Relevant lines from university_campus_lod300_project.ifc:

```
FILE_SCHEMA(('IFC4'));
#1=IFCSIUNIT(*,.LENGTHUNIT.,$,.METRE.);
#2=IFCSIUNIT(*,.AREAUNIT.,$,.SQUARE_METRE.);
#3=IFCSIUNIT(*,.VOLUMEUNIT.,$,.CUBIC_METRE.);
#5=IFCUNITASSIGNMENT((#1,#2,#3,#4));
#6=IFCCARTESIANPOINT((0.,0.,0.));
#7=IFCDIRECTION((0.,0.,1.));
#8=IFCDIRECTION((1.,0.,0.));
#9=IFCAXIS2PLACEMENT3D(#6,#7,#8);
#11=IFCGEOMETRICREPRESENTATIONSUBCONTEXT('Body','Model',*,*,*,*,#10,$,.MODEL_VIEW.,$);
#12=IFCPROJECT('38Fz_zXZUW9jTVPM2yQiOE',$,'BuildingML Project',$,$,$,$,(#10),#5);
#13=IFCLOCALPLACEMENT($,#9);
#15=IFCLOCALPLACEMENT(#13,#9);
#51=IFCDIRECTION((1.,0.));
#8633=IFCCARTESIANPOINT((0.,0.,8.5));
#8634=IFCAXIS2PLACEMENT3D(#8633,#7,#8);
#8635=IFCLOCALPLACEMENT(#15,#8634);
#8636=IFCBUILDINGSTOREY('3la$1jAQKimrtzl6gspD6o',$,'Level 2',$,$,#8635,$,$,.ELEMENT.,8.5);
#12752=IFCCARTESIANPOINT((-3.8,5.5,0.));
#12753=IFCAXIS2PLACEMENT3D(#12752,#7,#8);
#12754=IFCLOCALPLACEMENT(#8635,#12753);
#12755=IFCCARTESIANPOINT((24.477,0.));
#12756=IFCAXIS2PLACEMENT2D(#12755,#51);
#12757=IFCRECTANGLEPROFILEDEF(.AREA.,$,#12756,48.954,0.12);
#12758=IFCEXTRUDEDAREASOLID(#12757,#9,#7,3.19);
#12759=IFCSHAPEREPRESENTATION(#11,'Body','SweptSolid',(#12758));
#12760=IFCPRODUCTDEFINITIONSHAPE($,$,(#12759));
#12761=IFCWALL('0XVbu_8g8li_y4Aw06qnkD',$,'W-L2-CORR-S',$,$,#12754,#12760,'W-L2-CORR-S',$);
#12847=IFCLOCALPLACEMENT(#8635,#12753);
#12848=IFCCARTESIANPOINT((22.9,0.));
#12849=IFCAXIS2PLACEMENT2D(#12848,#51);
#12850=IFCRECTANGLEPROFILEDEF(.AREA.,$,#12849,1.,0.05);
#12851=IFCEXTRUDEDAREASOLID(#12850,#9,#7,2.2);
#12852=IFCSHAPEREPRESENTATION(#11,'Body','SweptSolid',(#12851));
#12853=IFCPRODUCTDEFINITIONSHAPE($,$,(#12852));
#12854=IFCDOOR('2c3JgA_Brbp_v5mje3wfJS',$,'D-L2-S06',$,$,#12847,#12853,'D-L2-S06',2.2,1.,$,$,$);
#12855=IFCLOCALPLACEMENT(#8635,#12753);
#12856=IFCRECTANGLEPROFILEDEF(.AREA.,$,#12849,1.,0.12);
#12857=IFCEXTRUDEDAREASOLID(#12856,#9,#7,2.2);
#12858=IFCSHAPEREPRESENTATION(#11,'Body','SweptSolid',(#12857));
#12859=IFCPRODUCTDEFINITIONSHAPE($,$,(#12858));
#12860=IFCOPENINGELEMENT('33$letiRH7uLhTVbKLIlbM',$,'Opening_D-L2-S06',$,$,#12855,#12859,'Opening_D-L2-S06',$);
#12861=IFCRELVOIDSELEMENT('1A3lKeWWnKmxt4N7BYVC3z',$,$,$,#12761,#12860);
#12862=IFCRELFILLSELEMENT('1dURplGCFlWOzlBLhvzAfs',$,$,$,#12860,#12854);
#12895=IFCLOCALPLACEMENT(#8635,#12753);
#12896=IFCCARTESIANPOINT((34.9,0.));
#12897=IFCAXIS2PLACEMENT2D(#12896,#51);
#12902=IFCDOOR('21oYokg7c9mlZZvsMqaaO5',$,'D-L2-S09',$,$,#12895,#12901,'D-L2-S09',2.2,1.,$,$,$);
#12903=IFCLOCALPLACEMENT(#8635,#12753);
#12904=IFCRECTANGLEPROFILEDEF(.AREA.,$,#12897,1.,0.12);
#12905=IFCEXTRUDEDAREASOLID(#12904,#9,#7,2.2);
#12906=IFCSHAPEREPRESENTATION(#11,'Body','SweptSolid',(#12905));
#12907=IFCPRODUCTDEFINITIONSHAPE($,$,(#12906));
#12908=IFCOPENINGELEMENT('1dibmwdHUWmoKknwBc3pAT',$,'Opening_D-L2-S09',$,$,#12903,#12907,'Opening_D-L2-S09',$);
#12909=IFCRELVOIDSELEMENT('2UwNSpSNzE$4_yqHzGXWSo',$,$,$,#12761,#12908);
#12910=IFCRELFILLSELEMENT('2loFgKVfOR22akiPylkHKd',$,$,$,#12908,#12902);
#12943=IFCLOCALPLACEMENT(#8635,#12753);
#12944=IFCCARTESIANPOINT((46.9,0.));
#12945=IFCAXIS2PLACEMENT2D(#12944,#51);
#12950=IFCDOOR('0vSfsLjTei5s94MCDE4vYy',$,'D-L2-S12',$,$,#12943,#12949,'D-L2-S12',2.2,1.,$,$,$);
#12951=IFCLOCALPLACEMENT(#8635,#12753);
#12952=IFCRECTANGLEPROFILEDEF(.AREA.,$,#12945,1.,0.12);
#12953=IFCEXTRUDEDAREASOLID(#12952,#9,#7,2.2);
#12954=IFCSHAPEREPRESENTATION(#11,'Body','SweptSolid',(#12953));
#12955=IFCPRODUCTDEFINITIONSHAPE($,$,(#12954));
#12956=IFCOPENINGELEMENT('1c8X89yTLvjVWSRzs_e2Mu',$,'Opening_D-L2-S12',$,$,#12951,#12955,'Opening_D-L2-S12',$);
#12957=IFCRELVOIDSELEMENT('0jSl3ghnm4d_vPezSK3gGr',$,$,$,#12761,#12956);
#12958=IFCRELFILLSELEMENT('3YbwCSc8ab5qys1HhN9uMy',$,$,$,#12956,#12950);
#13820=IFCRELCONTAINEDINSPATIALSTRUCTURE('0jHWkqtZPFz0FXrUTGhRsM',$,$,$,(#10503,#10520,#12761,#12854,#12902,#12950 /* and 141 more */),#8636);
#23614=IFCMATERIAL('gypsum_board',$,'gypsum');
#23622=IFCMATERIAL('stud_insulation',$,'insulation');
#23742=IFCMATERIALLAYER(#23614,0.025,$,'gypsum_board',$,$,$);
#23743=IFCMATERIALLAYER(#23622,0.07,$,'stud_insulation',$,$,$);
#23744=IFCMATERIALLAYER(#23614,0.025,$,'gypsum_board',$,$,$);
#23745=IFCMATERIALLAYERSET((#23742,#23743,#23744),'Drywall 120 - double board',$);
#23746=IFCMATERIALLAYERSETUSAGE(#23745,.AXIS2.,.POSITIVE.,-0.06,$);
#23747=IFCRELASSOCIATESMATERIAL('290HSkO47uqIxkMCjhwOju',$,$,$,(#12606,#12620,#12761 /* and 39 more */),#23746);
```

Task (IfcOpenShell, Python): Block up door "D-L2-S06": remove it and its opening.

```python
import ifcopenshell
import ifcopenshell.api.feature
import ifcopenshell.api.root
import ifcopenshell.geom
import ifcopenshell.util.shape

model = ifcopenshell.open("university_campus_lod300_project.ifc")
settings = ifcopenshell.geom.settings()


def volume(element):
    """Net volume in cubic metres, openings subtracted."""
    shape = ifcopenshell.geom.create_shape(settings, element)
    return ifcopenshell.util.shape.get_volume(shape.geometry)


door = model.by_id(12854)
opening = door.FillsVoids[0].RelatingOpeningElement
wall = opening.VoidsElements[0].RelatingBuildingElement
before = volume(wall)

ifcopenshell.api.root.remove_product(model, product=door)
ifcopenshell.api.feature.remove_feature(model, feature=opening)

after = volume(wall)

print(f"wall volume {before:.3f} -> {after:.3f} m3")

model.write("university_campus_lod300_project-out.ifc")
```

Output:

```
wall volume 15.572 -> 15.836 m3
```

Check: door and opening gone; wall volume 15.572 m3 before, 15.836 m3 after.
